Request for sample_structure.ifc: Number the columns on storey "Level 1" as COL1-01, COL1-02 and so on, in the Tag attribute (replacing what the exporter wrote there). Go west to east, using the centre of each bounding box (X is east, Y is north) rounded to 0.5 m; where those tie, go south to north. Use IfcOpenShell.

First a look at what the model holds.

```python
import ifcopenshell
import ifcopenshell.util.element
import ifcopenshell.util.placement

model = ifcopenshell.open("sample_structure.ifc")
print(model.schema)
storey = next(s for s in model.by_type("IfcBuildingStorey") if s.Name == "Level 1")
columns = [e for e in ifcopenshell.util.element.get_decomposition(storey) if e.is_a("IfcColumn")]
for e in sorted(columns, key=lambda e: e.id()):
    origin = ifcopenshell.util.placement.get_local_placement(e.ObjectPlacement)[:3, 3]
    print(e.id(), e.Tag, e.Name, origin.round(2) + 0.0, sep=" | ")
```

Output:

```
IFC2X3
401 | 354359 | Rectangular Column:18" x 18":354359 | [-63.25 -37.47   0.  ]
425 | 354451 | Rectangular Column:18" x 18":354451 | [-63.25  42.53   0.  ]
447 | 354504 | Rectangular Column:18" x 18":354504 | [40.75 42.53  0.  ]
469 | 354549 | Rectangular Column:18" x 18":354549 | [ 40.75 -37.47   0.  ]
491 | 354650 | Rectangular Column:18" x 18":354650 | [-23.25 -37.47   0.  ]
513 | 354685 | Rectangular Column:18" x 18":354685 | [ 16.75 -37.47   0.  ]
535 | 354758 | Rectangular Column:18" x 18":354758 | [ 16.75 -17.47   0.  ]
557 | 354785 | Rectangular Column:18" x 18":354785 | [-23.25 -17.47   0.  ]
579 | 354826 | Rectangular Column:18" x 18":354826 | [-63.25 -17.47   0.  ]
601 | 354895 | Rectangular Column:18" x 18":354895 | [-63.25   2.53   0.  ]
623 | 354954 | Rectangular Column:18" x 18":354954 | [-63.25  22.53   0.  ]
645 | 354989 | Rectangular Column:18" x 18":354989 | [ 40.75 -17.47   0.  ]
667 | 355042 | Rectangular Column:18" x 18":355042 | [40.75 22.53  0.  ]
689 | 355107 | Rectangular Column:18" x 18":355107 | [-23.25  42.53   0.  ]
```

```python
import ifcopenshell
import ifcopenshell.geom
import ifcopenshell.util.element
import ifcopenshell.util.shape

model = ifcopenshell.open("sample_structure.ifc")
settings = ifcopenshell.geom.settings()
settings.set("use-world-coords", True)


def centre(element):
    shape = ifcopenshell.geom.create_shape(settings, element)
    return ifcopenshell.util.shape.get_bbox_centroid(shape.geometry)


storey = next(s for s in model.by_type("IfcBuildingStorey") if s.Name == "Level 1")
columns = [e for e in ifcopenshell.util.element.get_decomposition(storey) if e.is_a("IfcColumn")]

# Insertion points can sit at a corner or the storey origin, so sort by the geometry (in metres).
centres = {e: centre(e) for e in columns}
columns.sort(key=lambda e: (round(centres[e][0] / 0.5), centres[e][1]))

for i, e in enumerate(columns, start=1):
    number = f"COL1-{i:02d}"
    e.Tag = number
    print(e.id(), number)

model.write("sample_structure_rev.ifc")
```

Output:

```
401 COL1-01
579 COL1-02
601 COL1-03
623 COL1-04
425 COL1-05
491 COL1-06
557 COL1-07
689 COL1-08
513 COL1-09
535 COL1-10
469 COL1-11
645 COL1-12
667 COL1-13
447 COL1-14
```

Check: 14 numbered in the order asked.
